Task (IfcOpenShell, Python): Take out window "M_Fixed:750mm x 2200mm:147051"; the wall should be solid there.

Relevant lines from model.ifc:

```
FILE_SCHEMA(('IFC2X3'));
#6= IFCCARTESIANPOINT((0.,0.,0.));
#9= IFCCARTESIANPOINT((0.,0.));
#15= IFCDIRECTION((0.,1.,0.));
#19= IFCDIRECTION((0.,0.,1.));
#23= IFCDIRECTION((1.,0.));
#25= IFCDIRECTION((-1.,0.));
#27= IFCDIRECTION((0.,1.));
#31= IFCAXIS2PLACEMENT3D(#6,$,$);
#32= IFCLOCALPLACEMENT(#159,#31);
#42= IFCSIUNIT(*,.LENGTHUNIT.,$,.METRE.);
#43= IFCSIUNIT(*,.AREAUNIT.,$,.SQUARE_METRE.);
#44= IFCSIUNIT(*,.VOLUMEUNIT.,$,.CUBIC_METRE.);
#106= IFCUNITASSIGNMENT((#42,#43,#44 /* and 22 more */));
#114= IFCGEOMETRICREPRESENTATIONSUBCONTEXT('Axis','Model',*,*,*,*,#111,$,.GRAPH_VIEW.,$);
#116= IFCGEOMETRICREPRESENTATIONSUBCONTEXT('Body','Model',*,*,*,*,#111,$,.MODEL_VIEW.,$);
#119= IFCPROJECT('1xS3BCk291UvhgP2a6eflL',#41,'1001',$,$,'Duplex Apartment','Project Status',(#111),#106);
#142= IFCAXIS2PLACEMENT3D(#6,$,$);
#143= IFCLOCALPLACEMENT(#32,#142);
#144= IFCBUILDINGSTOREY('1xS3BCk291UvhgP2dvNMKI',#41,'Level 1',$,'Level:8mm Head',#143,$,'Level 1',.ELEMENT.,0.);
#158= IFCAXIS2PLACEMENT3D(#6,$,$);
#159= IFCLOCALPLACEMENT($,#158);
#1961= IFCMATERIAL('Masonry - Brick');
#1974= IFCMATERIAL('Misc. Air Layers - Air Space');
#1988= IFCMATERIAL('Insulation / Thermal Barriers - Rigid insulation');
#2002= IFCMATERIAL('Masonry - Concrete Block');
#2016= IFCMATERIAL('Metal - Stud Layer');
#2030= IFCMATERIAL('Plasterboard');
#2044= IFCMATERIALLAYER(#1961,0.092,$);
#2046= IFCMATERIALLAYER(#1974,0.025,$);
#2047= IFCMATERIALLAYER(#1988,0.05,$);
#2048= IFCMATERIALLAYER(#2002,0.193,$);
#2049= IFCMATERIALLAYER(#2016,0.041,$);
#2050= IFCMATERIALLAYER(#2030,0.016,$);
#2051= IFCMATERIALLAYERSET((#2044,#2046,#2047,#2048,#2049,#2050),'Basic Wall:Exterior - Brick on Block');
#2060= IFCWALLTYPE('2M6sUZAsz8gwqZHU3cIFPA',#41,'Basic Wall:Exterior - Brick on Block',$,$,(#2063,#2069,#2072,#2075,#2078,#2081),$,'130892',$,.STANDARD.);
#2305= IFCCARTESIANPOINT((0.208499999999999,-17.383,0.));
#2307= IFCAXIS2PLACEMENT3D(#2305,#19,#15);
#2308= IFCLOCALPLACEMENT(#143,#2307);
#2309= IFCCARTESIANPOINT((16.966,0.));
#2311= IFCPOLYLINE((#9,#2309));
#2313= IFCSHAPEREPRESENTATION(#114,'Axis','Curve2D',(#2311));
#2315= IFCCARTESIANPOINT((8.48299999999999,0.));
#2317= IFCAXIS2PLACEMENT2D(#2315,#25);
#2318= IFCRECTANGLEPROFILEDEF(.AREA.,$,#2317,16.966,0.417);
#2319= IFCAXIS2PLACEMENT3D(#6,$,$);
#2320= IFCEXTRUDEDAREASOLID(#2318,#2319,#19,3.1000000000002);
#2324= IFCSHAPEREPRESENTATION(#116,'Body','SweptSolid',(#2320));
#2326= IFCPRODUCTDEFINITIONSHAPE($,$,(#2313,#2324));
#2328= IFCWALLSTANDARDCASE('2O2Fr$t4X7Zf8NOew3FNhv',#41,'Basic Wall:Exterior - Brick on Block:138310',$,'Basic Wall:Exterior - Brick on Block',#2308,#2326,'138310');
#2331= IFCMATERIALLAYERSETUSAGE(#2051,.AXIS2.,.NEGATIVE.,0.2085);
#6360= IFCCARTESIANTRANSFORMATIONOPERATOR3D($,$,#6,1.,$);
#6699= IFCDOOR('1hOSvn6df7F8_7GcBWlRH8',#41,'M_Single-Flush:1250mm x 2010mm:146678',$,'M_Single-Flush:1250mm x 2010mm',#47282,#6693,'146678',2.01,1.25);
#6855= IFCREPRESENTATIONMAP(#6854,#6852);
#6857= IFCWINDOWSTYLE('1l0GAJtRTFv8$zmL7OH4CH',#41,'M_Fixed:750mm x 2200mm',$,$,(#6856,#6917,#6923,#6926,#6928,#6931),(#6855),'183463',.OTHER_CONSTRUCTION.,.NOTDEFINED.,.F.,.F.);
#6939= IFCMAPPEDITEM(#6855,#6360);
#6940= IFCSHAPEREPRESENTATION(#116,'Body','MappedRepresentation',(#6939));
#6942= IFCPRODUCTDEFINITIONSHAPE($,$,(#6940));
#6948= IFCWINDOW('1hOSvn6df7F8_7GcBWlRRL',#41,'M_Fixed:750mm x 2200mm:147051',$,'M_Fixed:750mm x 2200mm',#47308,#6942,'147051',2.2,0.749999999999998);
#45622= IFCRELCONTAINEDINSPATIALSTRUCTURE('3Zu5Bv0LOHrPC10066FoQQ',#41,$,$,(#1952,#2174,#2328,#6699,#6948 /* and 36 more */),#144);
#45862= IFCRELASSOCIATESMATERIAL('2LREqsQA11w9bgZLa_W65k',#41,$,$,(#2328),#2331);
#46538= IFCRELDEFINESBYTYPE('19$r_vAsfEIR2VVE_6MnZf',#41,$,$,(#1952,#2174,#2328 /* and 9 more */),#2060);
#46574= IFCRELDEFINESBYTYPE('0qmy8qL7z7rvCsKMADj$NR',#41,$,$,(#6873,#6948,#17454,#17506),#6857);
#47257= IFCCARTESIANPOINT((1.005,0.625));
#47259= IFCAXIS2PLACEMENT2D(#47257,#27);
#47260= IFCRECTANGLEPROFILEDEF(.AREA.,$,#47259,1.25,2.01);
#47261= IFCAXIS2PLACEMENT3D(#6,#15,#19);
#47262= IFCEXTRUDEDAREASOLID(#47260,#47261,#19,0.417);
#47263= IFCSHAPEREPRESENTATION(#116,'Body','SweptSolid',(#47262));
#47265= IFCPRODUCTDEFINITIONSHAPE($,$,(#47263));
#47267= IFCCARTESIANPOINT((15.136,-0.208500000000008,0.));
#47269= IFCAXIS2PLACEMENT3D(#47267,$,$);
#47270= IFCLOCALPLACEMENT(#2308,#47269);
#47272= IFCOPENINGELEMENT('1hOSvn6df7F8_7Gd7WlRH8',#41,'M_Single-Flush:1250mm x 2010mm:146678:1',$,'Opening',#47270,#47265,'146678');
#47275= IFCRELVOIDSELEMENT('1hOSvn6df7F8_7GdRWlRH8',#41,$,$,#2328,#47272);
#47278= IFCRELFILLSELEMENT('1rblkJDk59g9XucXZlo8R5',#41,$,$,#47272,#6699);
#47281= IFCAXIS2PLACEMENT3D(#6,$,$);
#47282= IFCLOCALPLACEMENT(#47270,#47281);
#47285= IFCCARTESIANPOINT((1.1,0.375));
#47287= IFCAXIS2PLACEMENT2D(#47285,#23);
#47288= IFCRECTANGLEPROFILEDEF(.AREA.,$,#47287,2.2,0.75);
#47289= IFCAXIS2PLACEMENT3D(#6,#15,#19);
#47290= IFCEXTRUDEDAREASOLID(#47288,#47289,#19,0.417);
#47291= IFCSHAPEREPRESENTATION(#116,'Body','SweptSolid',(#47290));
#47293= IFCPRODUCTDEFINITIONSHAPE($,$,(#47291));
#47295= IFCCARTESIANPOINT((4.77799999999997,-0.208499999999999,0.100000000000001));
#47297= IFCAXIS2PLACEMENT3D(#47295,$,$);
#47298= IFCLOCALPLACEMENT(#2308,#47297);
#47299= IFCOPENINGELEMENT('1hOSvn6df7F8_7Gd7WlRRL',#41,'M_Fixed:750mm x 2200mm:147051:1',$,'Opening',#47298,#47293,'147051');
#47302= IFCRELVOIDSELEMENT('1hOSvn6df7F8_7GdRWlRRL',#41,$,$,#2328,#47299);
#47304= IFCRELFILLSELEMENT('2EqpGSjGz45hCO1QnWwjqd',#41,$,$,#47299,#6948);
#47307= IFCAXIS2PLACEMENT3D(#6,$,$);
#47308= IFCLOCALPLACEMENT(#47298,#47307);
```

```python
import ifcopenshell
import ifcopenshell.api.feature
import ifcopenshell.api.root
import ifcopenshell.geom
import ifcopenshell.util.shape

model = ifcopenshell.open("model.ifc")
settings = ifcopenshell.geom.settings()


def volume(element):
    """Net volume in cubic metres, openings subtracted."""
    shape = ifcopenshell.geom.create_shape(settings, element)
    return ifcopenshell.util.shape.get_volume(shape.geometry)


window = model.by_guid("1hOSvn6df7F8_7GcBWlRRL")
opening = window.FillsVoids[0].RelatingOpeningElement
wall = opening.VoidsElements[0].RelatingBuildingElement
before = volume(wall)

ifcopenshell.api.root.remove_product(model, product=window)
ifcopenshell.api.feature.remove_feature(model, feature=opening)

after = volume(wall)

print(f"wall volume {before:.3f} -> {after:.3f} m3")

model.write("model_edited.ifc")
```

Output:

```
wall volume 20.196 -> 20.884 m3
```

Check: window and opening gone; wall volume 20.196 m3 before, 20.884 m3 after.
